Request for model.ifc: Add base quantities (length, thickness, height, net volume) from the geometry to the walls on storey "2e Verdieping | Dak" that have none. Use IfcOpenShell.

First a look at what the model holds.

```python
import ifcopenshell
import ifcopenshell.util.element
import ifcopenshell.util.unit

model = ifcopenshell.open("model.ifc")
print(model.schema)
for unit_type in ("LENGTHUNIT", "AREAUNIT", "VOLUMEUNIT"):
    print(unit_type, ifcopenshell.util.unit.calculate_unit_scale(model, unit_type))
storey = next(s for s in model.by_type("IfcBuildingStorey") if s.Name == "2e Verdieping | Dak")
walls = [e for e in ifcopenshell.util.element.get_decomposition(storey) if e.is_a("IfcWall")]
for e in sorted(walls, key=lambda e: e.id()):
    print(e.id(), e.is_a(), e.Name, list(ifcopenshell.util.element.get_psets(e, qtos_only=True)), sep=" | ")
```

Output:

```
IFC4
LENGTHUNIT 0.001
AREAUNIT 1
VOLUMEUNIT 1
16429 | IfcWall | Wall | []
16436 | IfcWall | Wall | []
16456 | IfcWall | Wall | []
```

```python
import ifcopenshell
import ifcopenshell.api.pset
import ifcopenshell.geom
import ifcopenshell.util.element
import ifcopenshell.util.shape
import ifcopenshell.util.unit

model = ifcopenshell.open("model.ifc")
unit_scale = ifcopenshell.util.unit.calculate_unit_scale(model)
volume_scale = ifcopenshell.util.unit.calculate_unit_scale(model, "VOLUMEUNIT")
settings = ifcopenshell.geom.settings()

storey = next(s for s in model.by_type("IfcBuildingStorey") if s.Name == "2e Verdieping | Dak")
walls = [e for e in ifcopenshell.util.element.get_decomposition(storey) if e.is_a("IfcWall")]

for e in sorted(walls, key=lambda e: e.id()):
    if ifcopenshell.util.element.get_psets(e, qtos_only=True, should_inherit=False):
        continue
    # Geometry comes back in metres, in the element's own axes.
    shape = ifcopenshell.geom.create_shape(settings, e)
    values = {
        "Length": ifcopenshell.util.shape.get_x(shape.geometry) / unit_scale,
        "Width": ifcopenshell.util.shape.get_y(shape.geometry) / unit_scale,
        "Height": ifcopenshell.util.shape.get_z(shape.geometry) / unit_scale,
        "NetVolume": ifcopenshell.util.shape.get_volume(shape.geometry) / volume_scale,
    }
    qto = ifcopenshell.api.pset.add_qto(model, product=e, name="Qto_WallBaseQuantities")
    ifcopenshell.api.pset.edit_qto(model, qto=qto, properties=values)
    print(e.id(), {k: round(v, 3) for k, v in values.items()})

model.write("model_updated.ifc")
```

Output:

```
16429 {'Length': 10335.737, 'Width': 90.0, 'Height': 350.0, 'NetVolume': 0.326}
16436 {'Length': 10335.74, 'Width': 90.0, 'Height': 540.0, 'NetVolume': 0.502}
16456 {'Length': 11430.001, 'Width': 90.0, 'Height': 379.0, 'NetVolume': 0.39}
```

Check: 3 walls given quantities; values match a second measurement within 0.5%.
